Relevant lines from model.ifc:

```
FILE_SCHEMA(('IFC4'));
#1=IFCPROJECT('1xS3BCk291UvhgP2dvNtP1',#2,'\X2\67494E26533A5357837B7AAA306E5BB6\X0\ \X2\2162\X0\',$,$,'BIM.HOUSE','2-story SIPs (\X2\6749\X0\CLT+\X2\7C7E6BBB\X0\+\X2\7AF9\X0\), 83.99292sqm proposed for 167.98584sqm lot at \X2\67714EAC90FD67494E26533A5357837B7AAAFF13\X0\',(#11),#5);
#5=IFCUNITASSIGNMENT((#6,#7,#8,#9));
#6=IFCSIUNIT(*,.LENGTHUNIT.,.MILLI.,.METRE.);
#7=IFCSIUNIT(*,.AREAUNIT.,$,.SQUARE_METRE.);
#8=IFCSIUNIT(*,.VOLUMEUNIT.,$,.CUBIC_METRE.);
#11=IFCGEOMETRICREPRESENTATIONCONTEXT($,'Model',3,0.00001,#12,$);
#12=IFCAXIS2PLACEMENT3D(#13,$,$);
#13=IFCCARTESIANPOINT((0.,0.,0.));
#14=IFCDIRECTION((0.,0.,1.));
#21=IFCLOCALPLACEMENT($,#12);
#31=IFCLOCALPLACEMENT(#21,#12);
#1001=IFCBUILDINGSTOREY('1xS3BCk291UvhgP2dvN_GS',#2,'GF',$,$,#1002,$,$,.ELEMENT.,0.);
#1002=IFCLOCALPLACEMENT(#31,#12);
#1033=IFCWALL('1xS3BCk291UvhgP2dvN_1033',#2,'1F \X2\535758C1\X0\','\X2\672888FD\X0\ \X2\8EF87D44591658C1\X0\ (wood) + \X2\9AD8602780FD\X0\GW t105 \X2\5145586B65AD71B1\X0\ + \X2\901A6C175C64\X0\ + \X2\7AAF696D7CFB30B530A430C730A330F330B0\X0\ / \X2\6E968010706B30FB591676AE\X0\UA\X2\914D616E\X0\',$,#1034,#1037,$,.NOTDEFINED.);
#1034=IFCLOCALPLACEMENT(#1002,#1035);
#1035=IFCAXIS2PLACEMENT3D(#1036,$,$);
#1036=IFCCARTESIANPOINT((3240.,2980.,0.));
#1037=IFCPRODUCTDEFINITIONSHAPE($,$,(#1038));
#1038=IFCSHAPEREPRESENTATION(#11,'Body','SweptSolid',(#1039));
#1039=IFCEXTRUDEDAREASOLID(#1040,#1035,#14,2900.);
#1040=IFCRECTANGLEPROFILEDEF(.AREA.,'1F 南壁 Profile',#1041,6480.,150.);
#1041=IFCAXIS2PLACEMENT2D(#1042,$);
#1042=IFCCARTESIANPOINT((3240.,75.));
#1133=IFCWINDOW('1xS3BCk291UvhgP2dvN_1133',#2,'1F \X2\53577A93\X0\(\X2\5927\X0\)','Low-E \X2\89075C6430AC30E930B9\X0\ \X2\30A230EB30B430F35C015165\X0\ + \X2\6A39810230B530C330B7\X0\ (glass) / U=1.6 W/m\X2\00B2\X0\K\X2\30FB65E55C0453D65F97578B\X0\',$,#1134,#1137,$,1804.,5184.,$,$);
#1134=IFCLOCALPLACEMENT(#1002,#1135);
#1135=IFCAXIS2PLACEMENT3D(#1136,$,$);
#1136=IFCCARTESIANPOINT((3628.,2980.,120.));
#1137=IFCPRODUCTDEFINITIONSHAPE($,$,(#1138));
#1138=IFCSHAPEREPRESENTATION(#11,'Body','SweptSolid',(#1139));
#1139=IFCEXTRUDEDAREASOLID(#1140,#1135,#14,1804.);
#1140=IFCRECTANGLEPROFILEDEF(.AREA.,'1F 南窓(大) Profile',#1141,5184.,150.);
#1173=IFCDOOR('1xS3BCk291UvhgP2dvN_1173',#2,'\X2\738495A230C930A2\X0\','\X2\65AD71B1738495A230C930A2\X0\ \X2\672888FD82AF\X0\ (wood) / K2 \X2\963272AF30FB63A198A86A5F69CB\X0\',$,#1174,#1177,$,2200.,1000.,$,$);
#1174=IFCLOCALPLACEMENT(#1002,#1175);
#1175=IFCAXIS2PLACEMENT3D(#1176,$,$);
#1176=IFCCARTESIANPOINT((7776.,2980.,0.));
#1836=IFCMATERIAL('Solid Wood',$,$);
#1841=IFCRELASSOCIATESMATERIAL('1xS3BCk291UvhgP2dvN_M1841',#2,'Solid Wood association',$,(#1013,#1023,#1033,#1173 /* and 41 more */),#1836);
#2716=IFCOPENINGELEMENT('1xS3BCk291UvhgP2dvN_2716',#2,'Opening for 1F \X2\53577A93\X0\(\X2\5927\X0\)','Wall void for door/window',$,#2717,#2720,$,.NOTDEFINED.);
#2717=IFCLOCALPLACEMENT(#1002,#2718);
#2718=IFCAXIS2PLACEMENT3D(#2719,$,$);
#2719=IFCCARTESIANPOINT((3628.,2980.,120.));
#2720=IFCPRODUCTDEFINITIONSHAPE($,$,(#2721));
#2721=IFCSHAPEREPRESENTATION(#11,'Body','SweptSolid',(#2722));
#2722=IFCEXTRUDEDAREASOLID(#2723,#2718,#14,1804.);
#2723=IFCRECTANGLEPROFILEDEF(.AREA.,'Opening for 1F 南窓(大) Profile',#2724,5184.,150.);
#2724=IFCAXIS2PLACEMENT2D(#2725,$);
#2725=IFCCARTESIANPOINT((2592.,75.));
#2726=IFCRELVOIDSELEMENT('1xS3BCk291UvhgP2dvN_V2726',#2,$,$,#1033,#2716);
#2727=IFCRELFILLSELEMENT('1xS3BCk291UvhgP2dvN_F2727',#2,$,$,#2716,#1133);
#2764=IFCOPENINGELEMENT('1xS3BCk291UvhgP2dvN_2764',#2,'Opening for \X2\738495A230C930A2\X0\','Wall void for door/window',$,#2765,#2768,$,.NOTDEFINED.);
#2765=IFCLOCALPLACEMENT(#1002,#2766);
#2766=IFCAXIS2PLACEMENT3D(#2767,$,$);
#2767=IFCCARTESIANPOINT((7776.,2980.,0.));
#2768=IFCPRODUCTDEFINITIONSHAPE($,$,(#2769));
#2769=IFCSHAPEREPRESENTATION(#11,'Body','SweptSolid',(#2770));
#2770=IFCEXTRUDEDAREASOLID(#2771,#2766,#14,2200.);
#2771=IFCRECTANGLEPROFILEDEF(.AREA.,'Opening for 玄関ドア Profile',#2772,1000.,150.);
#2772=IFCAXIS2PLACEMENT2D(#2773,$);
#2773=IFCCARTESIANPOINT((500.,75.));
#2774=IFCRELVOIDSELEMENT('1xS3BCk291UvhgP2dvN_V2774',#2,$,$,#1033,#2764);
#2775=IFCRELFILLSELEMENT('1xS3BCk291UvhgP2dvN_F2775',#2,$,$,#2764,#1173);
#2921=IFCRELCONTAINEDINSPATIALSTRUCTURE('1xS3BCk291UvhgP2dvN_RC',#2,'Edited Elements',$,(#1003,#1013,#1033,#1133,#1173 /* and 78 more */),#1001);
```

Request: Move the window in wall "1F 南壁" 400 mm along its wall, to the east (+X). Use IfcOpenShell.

```python
import ifcopenshell
import ifcopenshell.api.geometry
import ifcopenshell.util.placement
import ifcopenshell.util.unit

model = ifcopenshell.open("model.ifc")
unit_scale = ifcopenshell.util.unit.calculate_unit_scale(model)

window = model.by_guid("1xS3BCk291UvhgP2dvN_1133")
opening = window.FillsVoids[0].RelatingOpeningElement
wall = opening.VoidsElements[0].RelatingBuildingElement

wall_matrix = ifcopenshell.util.placement.get_local_placement(wall.ObjectPlacement)
shift = wall_matrix[:3, 0] * 0.4 / unit_scale
before = ifcopenshell.util.placement.get_local_placement(window.ObjectPlacement)[:3, 3].copy()

# The window is not placed relative to its opening, so move both.
for product in (opening, window):
    matrix = ifcopenshell.util.placement.get_local_placement(product.ObjectPlacement)
    matrix[:3, 3] += shift
    ifcopenshell.api.geometry.edit_object_placement(model, product=product, matrix=matrix, is_si=False)

after = ifcopenshell.util.placement.get_local_placement(window.ObjectPlacement)[:3, 3]
print("window moved by", (after - before).round(3) + 0.0)

model.write("model_rev.ifc")
```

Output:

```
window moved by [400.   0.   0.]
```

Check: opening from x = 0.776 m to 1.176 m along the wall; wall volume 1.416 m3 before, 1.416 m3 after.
